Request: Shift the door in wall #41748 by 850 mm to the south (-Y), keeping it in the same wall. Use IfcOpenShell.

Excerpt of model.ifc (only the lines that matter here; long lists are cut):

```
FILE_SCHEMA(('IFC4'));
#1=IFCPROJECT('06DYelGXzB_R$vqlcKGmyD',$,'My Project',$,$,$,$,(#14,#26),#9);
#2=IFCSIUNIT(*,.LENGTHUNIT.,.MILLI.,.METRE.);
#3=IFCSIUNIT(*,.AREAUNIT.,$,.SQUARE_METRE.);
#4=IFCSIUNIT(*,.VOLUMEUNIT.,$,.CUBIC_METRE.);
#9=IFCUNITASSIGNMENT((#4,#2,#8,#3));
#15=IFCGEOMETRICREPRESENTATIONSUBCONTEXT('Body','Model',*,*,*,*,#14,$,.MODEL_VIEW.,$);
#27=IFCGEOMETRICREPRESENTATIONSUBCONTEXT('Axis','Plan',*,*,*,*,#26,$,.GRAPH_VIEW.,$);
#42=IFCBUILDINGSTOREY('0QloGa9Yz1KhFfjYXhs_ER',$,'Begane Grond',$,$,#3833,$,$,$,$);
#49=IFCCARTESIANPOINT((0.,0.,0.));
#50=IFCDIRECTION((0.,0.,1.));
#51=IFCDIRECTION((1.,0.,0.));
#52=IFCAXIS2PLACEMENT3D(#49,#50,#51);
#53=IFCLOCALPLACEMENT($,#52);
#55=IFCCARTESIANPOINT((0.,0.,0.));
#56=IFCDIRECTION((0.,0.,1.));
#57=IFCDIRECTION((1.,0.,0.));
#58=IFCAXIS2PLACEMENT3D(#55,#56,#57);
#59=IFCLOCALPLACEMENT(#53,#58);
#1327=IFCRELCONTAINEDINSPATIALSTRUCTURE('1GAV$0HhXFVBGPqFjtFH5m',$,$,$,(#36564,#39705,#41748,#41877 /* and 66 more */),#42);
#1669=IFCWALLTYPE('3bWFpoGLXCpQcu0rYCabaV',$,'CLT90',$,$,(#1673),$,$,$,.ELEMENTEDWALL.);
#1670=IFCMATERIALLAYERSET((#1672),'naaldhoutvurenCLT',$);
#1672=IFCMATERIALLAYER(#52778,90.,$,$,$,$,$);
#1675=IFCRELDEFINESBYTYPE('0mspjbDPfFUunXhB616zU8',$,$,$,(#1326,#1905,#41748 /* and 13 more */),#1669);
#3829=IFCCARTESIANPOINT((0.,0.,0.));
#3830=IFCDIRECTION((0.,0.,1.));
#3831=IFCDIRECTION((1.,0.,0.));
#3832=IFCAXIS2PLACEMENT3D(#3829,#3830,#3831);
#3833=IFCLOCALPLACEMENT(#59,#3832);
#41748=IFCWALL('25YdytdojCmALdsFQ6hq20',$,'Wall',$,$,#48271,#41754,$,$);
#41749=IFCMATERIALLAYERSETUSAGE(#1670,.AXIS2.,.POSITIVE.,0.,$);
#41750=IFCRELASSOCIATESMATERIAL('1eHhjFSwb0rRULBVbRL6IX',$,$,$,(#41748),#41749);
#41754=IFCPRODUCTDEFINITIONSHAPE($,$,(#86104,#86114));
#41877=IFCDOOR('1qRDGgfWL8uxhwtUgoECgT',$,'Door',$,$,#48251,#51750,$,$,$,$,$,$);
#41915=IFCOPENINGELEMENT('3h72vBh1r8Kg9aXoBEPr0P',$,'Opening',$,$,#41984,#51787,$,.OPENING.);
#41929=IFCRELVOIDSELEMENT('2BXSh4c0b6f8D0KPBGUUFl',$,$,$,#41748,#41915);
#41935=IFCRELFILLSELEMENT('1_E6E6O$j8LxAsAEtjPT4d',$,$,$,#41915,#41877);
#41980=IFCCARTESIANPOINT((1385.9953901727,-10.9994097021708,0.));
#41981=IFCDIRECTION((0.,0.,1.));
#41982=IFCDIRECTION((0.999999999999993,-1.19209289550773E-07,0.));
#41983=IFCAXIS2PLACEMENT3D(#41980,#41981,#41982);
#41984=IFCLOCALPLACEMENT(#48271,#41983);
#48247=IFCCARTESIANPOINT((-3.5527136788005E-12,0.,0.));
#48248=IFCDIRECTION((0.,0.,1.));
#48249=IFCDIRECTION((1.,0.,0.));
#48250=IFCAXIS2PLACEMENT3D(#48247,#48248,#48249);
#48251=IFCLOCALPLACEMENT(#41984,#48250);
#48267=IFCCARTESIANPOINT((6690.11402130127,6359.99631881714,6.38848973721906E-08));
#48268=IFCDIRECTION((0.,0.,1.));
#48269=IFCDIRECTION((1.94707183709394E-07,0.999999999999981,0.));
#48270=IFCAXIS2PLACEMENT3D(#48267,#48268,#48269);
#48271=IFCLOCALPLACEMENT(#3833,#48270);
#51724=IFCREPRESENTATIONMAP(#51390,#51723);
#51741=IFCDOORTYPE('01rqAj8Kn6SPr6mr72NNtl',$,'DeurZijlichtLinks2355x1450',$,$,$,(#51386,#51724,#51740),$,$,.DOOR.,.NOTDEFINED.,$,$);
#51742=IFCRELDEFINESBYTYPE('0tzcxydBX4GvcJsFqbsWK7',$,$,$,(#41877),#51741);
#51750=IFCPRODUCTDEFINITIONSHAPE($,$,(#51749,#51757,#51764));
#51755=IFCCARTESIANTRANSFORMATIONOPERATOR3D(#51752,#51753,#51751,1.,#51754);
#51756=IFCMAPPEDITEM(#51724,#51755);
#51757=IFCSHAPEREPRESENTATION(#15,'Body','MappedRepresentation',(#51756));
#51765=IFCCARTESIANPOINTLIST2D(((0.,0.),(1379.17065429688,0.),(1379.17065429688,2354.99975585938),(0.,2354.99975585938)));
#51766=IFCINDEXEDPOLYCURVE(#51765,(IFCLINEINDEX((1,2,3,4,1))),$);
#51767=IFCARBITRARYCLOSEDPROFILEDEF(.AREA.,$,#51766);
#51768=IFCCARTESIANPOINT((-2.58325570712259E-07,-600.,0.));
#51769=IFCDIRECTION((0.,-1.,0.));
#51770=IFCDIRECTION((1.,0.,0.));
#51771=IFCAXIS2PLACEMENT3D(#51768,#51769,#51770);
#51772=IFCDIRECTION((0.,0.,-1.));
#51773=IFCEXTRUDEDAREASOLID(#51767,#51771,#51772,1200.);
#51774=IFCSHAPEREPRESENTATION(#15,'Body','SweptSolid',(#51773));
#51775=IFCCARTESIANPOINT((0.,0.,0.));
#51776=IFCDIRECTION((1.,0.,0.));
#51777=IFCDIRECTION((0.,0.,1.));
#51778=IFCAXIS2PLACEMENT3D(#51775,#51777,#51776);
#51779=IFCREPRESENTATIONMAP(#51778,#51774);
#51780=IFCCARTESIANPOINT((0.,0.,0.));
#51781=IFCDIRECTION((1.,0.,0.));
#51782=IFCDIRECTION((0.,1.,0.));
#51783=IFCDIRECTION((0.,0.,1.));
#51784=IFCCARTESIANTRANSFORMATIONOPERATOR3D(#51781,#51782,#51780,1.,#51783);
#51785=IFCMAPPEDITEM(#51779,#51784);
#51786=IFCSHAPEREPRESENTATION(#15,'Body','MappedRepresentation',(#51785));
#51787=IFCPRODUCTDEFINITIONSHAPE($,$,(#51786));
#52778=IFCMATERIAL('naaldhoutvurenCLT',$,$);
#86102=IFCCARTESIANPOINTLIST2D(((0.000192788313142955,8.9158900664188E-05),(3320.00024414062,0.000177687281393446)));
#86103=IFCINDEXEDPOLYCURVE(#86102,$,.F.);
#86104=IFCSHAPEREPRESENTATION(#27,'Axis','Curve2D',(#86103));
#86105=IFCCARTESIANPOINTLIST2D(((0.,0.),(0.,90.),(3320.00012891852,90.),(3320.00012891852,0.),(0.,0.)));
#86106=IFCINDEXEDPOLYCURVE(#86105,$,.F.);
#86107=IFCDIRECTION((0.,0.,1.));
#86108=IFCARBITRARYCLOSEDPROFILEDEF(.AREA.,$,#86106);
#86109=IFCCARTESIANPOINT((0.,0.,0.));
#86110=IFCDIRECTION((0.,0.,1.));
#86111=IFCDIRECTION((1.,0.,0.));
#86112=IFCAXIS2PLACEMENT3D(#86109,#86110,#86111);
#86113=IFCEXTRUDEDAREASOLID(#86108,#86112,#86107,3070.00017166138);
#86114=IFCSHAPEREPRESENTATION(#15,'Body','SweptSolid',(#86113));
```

```python
import ifcopenshell
import ifcopenshell.api.geometry
import ifcopenshell.util.placement
import ifcopenshell.util.unit

model = ifcopenshell.open("model.ifc")
unit_scale = ifcopenshell.util.unit.calculate_unit_scale(model)

door = model.by_guid("1qRDGgfWL8uxhwtUgoECgT")
opening = door.FillsVoids[0].RelatingOpeningElement
wall = opening.VoidsElements[0].RelatingBuildingElement

wall_matrix = ifcopenshell.util.placement.get_local_placement(wall.ObjectPlacement)
shift = wall_matrix[:3, 0] * -0.85 / unit_scale
before = ifcopenshell.util.placement.get_local_placement(door.ObjectPlacement)[:3, 3].copy()

# The door is placed relative to its opening, so it follows when the opening moves.
matrix = ifcopenshell.util.placement.get_local_placement(opening.ObjectPlacement)
matrix[:3, 3] += shift
ifcopenshell.api.geometry.edit_object_placement(
    model, product=opening, matrix=matrix, is_si=False, should_transform_children=True
)

after = ifcopenshell.util.placement.get_local_placement(door.ObjectPlacement)[:3, 3]
print("door moved by", (after - before).round(3) + 0.0)

model.write("model_edited.ifc")
```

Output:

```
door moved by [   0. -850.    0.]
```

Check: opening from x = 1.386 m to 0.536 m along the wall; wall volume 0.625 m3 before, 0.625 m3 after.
